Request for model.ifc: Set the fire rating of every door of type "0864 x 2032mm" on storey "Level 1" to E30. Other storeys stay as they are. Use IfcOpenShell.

First a look at what the model holds.

```python
import ifcopenshell
import ifcopenshell.util.element

model = ifcopenshell.open("model.ifc")
print(model.schema)
storey = next(s for s in model.by_type("IfcBuildingStorey") if s.Name == "Level 1")
doors = [e for e in ifcopenshell.util.element.get_decomposition(storey) if e.is_a("IfcDoor")]
seen = {}
for e in doors:
    element_type = ifcopenshell.util.element.get_type(e)
    key = (element_type.Name if element_type != e and element_type else None, ifcopenshell.util.element.get_pset(e, "Pset_DoorCommon", "FireRating"))
    seen[key] = seen.get(key, 0) + 1
for (name, value), count in sorted(seen.items(), key=str):
    print(count, "x", name, "|", value)
```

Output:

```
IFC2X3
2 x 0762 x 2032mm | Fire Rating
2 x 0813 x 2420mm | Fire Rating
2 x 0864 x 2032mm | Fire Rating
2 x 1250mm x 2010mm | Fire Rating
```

```python
import ifcopenshell
import ifcopenshell.api.pset
import ifcopenshell.util.element

model = ifcopenshell.open("model.ifc")

storey = next(s for s in model.by_type("IfcBuildingStorey") if s.Name == "Level 1")
doors = [e for e in ifcopenshell.util.element.get_decomposition(storey) if e.is_a("IfcDoor")]

count = 0
for e in doors:
    element_type = ifcopenshell.util.element.get_type(e)
    if element_type in (None, e) or element_type.Name != "0864 x 2032mm":
        continue
    # add_pset returns the element's existing set when there is one.
    pset = ifcopenshell.api.pset.add_pset(model, product=e, name="Pset_DoorCommon")
    ifcopenshell.api.pset.edit_pset(model, pset=pset, properties={"FireRating": "E30"})
    count += 1

print(count, "doors updated")

model.write("model_v2.ifc")
```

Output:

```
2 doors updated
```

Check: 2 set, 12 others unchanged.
